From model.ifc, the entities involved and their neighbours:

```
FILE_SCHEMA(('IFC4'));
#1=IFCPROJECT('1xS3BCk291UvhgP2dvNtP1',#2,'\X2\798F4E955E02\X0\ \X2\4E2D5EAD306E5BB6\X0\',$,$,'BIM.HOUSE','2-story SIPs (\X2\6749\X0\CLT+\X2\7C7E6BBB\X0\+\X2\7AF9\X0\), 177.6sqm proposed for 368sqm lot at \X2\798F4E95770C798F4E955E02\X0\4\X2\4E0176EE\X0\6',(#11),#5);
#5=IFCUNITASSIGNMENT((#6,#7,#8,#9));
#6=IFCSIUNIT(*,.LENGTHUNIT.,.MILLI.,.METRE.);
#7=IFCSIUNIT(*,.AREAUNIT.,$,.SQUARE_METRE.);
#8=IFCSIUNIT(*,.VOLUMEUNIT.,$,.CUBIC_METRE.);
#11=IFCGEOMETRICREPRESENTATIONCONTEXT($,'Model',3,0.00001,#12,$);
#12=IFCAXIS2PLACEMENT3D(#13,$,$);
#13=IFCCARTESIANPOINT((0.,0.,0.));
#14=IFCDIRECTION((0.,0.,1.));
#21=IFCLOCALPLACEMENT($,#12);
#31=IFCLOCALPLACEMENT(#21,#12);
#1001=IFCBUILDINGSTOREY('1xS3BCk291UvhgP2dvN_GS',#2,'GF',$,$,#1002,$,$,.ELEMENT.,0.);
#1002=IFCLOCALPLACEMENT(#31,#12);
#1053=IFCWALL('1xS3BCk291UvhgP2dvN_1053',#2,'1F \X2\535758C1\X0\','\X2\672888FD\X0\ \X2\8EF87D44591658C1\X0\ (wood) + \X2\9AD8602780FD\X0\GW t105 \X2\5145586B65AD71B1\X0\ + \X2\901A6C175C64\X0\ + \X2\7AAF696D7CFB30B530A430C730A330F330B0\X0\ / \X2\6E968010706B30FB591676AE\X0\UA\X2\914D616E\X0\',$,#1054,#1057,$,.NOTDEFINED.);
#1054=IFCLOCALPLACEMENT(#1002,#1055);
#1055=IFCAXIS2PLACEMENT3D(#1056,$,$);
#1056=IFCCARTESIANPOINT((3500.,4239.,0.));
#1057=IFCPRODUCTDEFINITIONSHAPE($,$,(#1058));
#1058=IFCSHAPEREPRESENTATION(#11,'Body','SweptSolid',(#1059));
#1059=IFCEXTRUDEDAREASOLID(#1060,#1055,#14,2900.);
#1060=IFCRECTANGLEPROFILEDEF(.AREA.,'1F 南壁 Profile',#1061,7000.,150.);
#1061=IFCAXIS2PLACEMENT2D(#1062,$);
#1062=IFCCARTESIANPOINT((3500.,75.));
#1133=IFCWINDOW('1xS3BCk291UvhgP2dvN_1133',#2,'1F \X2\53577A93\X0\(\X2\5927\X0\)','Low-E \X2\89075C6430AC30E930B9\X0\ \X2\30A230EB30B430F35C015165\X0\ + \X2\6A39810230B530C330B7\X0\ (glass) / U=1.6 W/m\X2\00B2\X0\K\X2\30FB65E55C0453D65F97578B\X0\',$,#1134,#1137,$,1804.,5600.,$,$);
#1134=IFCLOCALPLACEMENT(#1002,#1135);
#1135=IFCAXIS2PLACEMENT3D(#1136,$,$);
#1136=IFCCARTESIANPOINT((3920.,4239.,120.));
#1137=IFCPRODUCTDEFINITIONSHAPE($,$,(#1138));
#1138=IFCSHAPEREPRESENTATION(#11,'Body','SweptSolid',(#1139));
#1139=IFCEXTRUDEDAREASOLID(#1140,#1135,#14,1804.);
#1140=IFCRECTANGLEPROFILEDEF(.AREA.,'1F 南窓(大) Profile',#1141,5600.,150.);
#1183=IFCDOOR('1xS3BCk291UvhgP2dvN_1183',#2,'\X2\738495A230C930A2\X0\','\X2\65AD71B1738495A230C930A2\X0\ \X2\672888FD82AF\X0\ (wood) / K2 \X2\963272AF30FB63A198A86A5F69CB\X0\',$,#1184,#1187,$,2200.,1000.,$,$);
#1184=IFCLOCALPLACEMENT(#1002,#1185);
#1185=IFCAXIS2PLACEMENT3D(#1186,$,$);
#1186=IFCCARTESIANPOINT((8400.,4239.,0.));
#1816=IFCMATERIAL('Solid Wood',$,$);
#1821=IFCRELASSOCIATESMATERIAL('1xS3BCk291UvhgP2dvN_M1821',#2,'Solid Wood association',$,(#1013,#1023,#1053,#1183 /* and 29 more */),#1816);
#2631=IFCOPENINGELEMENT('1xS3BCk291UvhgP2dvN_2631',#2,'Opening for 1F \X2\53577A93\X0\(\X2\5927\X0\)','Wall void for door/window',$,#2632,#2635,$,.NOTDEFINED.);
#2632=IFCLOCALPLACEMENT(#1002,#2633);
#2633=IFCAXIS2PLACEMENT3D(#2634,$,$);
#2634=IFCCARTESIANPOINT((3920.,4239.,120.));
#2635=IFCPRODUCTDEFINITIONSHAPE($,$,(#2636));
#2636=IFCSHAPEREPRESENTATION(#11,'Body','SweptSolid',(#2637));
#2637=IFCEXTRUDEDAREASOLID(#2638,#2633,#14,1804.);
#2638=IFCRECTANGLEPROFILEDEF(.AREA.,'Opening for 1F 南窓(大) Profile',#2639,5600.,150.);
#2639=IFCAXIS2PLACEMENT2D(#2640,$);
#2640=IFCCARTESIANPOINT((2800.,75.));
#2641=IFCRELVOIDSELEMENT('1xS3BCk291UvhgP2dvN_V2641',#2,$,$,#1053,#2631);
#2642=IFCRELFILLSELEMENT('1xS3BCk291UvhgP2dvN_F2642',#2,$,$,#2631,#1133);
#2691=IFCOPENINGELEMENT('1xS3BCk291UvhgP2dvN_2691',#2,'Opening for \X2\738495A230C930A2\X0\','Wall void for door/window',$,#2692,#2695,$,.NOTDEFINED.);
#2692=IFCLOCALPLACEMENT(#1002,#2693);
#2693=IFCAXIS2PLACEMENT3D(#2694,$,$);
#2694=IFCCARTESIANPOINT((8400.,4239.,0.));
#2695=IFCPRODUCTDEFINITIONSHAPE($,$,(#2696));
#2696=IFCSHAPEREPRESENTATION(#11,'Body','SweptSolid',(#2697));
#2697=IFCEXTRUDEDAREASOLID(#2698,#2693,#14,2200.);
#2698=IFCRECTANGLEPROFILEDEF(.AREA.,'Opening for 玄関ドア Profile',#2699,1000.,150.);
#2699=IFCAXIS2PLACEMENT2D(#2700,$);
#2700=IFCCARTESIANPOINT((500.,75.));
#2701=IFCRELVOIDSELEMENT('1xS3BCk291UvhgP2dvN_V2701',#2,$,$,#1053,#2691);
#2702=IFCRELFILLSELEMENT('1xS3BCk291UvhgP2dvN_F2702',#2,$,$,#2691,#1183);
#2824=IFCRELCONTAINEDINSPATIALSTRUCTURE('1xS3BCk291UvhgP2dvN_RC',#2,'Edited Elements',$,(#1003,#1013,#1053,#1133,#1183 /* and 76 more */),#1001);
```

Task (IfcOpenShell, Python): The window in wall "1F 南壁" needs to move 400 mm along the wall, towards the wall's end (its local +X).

```python
import ifcopenshell
import ifcopenshell.api.geometry
import ifcopenshell.util.placement

model = ifcopenshell.open("model.ifc")

window = model.by_guid("1xS3BCk291UvhgP2dvN_1133")
opening = window.FillsVoids[0].RelatingOpeningElement
wall = opening.VoidsElements[0].RelatingBuildingElement

wall_matrix = ifcopenshell.util.placement.get_local_placement(wall.ObjectPlacement)
shift = wall_matrix[:3, 0] * 400.0
before = ifcopenshell.util.placement.get_local_placement(window.ObjectPlacement)[:3, 3].copy()

# The window is not placed relative to its opening, so move both.
for product in (opening, window):
    matrix = ifcopenshell.util.placement.get_local_placement(product.ObjectPlacement)
    matrix[:3, 3] += shift
    ifcopenshell.api.geometry.edit_object_placement(model, product=product, matrix=matrix, is_si=False)

after = ifcopenshell.util.placement.get_local_placement(window.ObjectPlacement)[:3, 3]
print("window moved by", (after - before).round(3) + 0.0)

model.write("model_v2.ifc")
```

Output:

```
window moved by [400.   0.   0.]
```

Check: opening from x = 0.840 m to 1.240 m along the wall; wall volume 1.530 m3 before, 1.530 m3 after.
